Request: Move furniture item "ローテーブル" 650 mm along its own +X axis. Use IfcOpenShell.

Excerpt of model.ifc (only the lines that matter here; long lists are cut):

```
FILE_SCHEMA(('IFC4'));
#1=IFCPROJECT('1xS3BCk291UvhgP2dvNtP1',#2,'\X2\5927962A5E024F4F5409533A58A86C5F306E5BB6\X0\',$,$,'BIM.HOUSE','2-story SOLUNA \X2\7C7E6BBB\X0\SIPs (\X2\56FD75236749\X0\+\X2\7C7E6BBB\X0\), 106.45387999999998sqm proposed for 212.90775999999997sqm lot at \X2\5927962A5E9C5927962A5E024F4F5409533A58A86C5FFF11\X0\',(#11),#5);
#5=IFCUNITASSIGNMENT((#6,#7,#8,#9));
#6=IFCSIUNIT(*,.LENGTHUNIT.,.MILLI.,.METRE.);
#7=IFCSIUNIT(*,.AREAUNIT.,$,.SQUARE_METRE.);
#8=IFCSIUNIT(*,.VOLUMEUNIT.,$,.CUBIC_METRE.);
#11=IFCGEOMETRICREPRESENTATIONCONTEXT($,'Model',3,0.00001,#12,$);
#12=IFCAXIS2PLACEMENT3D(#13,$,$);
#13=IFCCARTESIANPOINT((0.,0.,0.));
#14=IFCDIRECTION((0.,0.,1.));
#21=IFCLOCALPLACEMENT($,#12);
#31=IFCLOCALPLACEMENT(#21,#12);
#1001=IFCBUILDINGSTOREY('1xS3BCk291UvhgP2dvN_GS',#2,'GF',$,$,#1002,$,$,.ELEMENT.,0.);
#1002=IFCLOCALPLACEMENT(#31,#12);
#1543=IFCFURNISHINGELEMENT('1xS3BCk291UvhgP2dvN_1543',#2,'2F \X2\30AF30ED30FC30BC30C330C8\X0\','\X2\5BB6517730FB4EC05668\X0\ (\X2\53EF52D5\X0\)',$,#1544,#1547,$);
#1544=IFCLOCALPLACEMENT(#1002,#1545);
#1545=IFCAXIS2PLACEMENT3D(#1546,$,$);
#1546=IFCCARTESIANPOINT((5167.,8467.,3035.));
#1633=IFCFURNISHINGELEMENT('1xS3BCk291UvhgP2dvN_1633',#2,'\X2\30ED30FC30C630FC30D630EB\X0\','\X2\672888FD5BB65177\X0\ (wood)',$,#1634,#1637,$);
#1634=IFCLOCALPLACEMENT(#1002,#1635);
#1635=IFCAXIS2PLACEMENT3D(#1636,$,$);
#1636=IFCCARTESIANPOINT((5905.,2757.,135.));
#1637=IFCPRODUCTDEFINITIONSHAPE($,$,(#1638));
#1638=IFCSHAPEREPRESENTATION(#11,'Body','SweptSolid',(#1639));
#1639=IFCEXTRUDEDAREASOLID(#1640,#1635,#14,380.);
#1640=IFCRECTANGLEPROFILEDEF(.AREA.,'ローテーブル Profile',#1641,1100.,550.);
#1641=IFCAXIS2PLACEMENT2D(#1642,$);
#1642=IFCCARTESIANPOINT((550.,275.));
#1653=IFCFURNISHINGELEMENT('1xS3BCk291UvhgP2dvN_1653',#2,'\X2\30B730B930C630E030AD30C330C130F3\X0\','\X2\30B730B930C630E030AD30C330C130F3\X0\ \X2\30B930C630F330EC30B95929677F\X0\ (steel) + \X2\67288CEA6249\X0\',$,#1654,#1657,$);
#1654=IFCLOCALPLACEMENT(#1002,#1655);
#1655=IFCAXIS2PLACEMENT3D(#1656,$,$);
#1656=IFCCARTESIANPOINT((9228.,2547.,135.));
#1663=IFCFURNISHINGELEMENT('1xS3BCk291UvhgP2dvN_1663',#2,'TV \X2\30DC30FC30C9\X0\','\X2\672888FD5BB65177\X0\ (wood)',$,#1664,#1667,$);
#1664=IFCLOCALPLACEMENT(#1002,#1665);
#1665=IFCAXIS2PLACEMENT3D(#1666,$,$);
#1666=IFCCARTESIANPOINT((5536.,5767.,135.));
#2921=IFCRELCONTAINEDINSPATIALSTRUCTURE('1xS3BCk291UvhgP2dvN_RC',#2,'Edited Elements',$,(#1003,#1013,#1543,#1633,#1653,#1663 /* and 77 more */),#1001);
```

```python
import ifcopenshell
import ifcopenshell.api.geometry
import ifcopenshell.util.placement
import ifcopenshell.util.unit

model = ifcopenshell.open("model.ifc")
unit_scale = ifcopenshell.util.unit.calculate_unit_scale(model)

item = model.by_guid("1xS3BCk291UvhgP2dvN_1633")
matrix = ifcopenshell.util.placement.get_local_placement(item.ObjectPlacement)
matrix[:3, 3] += matrix[:3, 0] * 0.65 / unit_scale
ifcopenshell.api.geometry.edit_object_placement(model, product=item, matrix=matrix, is_si=False)

print(ifcopenshell.util.placement.get_local_placement(item.ObjectPlacement).round(3) + 0.0)

model.write("model_updated.ifc")
```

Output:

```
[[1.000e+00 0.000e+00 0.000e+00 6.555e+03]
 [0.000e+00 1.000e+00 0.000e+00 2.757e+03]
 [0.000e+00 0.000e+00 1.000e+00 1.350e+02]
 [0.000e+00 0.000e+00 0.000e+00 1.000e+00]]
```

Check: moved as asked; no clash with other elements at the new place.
